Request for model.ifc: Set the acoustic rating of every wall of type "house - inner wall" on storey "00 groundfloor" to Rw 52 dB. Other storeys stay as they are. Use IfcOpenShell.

First a look at what the model holds.

```python
import ifcopenshell
import ifcopenshell.util.element

model = ifcopenshell.open("model.ifc")
print(model.schema)
storey = next(s for s in model.by_type("IfcBuildingStorey") if s.Name == "00 groundfloor")
walls = [e for e in ifcopenshell.util.element.get_decomposition(storey) if e.is_a("IfcWall")]
seen = {}
for e in walls:
    element_type = ifcopenshell.util.element.get_type(e)
    key = (element_type.Name if element_type != e and element_type else None, ifcopenshell.util.element.get_pset(e, "Pset_WallCommon", "AcousticRating"))
    seen[key] = seen.get(key, 0) + 1
for (name, value), count in sorted(seen.items(), key=str):
    print(count, "x", name, "|", value)
```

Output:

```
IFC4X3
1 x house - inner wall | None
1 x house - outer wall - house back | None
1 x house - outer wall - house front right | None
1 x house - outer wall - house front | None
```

```python
import ifcopenshell
import ifcopenshell.api.pset
import ifcopenshell.util.element

model = ifcopenshell.open("model.ifc")

storey = next(s for s in model.by_type("IfcBuildingStorey") if s.Name == "00 groundfloor")
walls = [e for e in ifcopenshell.util.element.get_decomposition(storey) if e.is_a("IfcWall")]

count = 0
for e in walls:
    element_type = ifcopenshell.util.element.get_type(e)
    if element_type in (None, e) or element_type.Name != "house - inner wall":
        continue
    # add_pset returns the element's existing set when there is one.
    pset = ifcopenshell.api.pset.add_pset(model, product=e, name="Pset_WallCommon")
    ifcopenshell.api.pset.edit_pset(model, pset=pset, properties={"AcousticRating": "Rw 52 dB"})
    count += 1

print(count, "walls updated")

model.write("model-out.ifc")
```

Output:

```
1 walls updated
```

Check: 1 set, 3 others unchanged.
